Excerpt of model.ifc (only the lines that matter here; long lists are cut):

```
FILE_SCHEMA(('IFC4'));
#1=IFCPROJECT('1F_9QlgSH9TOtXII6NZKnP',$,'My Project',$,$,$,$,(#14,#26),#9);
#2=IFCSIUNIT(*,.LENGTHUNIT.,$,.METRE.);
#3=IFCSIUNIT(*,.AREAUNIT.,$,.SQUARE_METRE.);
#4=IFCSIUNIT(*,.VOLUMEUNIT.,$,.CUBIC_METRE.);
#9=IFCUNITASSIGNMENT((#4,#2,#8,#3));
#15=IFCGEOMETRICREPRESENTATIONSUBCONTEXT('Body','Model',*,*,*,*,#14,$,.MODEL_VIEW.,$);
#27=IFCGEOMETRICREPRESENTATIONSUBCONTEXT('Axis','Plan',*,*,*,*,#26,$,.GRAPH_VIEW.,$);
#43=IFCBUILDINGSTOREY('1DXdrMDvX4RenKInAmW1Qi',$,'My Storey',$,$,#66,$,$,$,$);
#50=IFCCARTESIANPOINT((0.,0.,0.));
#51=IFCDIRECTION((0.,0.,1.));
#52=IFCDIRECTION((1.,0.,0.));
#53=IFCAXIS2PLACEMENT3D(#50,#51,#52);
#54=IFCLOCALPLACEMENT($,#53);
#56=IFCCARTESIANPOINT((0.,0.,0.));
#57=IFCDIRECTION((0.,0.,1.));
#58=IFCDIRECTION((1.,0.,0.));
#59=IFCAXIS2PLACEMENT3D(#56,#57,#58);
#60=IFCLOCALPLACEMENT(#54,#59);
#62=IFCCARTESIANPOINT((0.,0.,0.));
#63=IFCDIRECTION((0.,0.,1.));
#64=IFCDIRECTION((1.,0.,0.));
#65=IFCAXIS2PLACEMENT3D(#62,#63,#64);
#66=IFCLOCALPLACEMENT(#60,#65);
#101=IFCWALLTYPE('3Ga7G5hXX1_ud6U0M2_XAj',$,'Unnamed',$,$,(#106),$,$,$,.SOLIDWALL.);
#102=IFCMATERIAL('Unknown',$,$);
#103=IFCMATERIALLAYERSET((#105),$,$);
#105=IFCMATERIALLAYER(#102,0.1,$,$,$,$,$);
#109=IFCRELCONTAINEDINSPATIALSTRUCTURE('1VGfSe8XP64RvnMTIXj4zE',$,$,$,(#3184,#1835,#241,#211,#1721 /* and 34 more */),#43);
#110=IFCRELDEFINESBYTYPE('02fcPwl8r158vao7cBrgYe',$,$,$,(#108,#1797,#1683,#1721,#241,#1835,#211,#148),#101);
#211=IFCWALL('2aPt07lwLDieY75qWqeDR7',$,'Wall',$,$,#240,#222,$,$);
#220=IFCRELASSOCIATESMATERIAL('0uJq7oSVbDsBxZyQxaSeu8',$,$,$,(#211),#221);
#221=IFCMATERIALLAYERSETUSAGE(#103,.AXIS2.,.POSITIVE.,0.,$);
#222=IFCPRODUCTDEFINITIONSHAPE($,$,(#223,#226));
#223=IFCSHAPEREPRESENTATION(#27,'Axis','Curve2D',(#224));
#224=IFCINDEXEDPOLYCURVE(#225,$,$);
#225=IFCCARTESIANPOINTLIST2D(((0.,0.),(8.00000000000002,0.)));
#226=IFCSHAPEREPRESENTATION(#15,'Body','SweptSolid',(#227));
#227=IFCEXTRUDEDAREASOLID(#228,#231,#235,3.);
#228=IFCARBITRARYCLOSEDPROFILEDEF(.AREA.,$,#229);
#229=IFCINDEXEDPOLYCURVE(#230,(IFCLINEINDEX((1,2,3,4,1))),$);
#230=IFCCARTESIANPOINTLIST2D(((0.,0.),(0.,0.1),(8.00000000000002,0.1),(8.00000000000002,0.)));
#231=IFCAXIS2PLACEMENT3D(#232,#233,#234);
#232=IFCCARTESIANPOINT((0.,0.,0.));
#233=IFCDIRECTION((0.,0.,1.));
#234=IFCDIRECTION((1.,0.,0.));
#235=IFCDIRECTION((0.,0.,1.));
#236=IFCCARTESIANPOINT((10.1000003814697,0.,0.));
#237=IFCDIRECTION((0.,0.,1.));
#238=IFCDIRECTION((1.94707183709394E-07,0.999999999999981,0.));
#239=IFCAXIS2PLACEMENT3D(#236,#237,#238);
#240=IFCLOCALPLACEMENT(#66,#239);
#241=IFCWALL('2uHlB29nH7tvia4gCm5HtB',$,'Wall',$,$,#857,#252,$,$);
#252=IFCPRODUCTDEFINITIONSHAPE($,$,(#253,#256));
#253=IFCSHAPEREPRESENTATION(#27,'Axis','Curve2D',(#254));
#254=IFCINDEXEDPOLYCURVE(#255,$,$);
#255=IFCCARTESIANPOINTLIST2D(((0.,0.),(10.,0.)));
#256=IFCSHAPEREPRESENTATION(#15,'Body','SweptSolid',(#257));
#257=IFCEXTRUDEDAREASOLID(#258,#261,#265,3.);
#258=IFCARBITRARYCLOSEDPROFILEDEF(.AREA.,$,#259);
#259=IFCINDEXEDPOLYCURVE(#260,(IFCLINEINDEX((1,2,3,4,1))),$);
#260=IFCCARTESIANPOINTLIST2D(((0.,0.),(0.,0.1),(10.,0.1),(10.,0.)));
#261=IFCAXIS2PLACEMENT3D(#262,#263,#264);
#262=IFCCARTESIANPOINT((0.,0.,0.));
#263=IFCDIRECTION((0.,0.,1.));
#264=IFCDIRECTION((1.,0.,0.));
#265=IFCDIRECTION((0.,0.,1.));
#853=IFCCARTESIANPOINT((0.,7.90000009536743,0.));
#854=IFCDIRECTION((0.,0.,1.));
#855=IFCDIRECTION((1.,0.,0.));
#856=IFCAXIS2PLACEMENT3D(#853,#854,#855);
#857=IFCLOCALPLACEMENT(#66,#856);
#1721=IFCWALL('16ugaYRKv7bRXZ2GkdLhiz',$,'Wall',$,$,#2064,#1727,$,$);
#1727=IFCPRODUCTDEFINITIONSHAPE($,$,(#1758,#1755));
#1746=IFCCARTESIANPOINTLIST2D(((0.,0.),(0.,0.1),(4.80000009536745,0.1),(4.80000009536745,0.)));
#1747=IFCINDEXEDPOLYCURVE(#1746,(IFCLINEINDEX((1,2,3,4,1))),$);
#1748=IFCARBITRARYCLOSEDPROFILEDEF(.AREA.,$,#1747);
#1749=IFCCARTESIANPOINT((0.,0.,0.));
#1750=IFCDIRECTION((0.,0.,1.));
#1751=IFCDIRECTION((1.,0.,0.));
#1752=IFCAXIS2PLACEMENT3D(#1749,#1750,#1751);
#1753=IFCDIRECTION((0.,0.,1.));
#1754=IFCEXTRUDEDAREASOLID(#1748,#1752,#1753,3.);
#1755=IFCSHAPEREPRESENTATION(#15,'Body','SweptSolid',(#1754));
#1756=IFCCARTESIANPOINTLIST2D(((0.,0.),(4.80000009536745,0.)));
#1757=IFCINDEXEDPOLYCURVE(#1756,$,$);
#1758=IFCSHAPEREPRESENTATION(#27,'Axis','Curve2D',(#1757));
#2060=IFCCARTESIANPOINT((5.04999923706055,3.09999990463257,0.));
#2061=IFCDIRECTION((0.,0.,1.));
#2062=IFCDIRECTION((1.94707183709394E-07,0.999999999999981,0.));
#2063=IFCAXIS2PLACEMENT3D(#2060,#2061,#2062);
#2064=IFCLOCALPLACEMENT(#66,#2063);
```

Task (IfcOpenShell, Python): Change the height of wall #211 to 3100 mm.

```python
import ifcopenshell
import ifcopenshell.geom
import ifcopenshell.util.representation
import ifcopenshell.util.shape

model = ifcopenshell.open("model.ifc")
settings = ifcopenshell.geom.settings()


def volume(element):
    """Net volume in cubic metres, openings subtracted."""
    shape = ifcopenshell.geom.create_shape(settings, element)
    return ifcopenshell.util.shape.get_volume(shape.geometry)


wall = model.by_id(211)
before = volume(wall)

body = ifcopenshell.util.representation.get_representation(wall, "Model", "Body")
solid = body.Items[0]
old_height = solid.Depth
solid.Depth = 3.1
after = volume(wall)

print(f"height {old_height:g} -> {solid.Depth:g}, volume {before:.3f} -> {after:.3f} m3")

model.write("model_rev.ifc")
```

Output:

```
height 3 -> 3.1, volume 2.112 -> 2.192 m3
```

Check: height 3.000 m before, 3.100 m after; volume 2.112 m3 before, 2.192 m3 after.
